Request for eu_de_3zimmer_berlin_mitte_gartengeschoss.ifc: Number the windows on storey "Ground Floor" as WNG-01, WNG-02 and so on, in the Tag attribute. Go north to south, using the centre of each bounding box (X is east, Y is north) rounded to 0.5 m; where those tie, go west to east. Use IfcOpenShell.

First a look at what the model holds.

```python
import ifcopenshell
import ifcopenshell.util.element
import ifcopenshell.util.placement

model = ifcopenshell.open("eu_de_3zimmer_berlin_mitte_gartengeschoss.ifc")
print(model.schema)
storey = next(s for s in model.by_type("IfcBuildingStorey") if s.Name == "Ground Floor")
windows = [e for e in ifcopenshell.util.element.get_decomposition(storey) if e.is_a("IfcWindow")]
for e in sorted(windows, key=lambda e: e.id()):
    origin = ifcopenshell.util.placement.get_local_placement(e.ObjectPlacement)[:3, 3]
    print(e.id(), e.Tag, e.Name, origin.round(2) + 0.0, sep=" | ")
```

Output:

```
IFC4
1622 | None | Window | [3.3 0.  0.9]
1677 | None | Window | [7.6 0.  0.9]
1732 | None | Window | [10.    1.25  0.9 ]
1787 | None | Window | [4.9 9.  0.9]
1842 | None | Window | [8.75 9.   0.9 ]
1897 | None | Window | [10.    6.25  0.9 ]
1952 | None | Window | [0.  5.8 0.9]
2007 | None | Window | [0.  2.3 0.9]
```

```python
import ifcopenshell
import ifcopenshell.geom
import ifcopenshell.util.element
import ifcopenshell.util.shape

model = ifcopenshell.open("eu_de_3zimmer_berlin_mitte_gartengeschoss.ifc")
settings = ifcopenshell.geom.settings()
settings.set("use-world-coords", True)


def centre(element):
    shape = ifcopenshell.geom.create_shape(settings, element)
    return ifcopenshell.util.shape.get_bbox_centroid(shape.geometry)


storey = next(s for s in model.by_type("IfcBuildingStorey") if s.Name == "Ground Floor")
windows = [e for e in ifcopenshell.util.element.get_decomposition(storey) if e.is_a("IfcWindow")]

# Insertion points can sit at a corner or the storey origin, so sort by the geometry (in metres).
centres = {e: centre(e) for e in windows}
windows.sort(key=lambda e: (-round(centres[e][1] / 0.5), centres[e][0]))

for i, e in enumerate(windows, start=1):
    number = f"WNG-{i:02d}"
    e.Tag = number
    print(e.id(), number)

model.write("eu_de_3zimmer_berlin_mitte_gartengeschoss_updated.ifc")
```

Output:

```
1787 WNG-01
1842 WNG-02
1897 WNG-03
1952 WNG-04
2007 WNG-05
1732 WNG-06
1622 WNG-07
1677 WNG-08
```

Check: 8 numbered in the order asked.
